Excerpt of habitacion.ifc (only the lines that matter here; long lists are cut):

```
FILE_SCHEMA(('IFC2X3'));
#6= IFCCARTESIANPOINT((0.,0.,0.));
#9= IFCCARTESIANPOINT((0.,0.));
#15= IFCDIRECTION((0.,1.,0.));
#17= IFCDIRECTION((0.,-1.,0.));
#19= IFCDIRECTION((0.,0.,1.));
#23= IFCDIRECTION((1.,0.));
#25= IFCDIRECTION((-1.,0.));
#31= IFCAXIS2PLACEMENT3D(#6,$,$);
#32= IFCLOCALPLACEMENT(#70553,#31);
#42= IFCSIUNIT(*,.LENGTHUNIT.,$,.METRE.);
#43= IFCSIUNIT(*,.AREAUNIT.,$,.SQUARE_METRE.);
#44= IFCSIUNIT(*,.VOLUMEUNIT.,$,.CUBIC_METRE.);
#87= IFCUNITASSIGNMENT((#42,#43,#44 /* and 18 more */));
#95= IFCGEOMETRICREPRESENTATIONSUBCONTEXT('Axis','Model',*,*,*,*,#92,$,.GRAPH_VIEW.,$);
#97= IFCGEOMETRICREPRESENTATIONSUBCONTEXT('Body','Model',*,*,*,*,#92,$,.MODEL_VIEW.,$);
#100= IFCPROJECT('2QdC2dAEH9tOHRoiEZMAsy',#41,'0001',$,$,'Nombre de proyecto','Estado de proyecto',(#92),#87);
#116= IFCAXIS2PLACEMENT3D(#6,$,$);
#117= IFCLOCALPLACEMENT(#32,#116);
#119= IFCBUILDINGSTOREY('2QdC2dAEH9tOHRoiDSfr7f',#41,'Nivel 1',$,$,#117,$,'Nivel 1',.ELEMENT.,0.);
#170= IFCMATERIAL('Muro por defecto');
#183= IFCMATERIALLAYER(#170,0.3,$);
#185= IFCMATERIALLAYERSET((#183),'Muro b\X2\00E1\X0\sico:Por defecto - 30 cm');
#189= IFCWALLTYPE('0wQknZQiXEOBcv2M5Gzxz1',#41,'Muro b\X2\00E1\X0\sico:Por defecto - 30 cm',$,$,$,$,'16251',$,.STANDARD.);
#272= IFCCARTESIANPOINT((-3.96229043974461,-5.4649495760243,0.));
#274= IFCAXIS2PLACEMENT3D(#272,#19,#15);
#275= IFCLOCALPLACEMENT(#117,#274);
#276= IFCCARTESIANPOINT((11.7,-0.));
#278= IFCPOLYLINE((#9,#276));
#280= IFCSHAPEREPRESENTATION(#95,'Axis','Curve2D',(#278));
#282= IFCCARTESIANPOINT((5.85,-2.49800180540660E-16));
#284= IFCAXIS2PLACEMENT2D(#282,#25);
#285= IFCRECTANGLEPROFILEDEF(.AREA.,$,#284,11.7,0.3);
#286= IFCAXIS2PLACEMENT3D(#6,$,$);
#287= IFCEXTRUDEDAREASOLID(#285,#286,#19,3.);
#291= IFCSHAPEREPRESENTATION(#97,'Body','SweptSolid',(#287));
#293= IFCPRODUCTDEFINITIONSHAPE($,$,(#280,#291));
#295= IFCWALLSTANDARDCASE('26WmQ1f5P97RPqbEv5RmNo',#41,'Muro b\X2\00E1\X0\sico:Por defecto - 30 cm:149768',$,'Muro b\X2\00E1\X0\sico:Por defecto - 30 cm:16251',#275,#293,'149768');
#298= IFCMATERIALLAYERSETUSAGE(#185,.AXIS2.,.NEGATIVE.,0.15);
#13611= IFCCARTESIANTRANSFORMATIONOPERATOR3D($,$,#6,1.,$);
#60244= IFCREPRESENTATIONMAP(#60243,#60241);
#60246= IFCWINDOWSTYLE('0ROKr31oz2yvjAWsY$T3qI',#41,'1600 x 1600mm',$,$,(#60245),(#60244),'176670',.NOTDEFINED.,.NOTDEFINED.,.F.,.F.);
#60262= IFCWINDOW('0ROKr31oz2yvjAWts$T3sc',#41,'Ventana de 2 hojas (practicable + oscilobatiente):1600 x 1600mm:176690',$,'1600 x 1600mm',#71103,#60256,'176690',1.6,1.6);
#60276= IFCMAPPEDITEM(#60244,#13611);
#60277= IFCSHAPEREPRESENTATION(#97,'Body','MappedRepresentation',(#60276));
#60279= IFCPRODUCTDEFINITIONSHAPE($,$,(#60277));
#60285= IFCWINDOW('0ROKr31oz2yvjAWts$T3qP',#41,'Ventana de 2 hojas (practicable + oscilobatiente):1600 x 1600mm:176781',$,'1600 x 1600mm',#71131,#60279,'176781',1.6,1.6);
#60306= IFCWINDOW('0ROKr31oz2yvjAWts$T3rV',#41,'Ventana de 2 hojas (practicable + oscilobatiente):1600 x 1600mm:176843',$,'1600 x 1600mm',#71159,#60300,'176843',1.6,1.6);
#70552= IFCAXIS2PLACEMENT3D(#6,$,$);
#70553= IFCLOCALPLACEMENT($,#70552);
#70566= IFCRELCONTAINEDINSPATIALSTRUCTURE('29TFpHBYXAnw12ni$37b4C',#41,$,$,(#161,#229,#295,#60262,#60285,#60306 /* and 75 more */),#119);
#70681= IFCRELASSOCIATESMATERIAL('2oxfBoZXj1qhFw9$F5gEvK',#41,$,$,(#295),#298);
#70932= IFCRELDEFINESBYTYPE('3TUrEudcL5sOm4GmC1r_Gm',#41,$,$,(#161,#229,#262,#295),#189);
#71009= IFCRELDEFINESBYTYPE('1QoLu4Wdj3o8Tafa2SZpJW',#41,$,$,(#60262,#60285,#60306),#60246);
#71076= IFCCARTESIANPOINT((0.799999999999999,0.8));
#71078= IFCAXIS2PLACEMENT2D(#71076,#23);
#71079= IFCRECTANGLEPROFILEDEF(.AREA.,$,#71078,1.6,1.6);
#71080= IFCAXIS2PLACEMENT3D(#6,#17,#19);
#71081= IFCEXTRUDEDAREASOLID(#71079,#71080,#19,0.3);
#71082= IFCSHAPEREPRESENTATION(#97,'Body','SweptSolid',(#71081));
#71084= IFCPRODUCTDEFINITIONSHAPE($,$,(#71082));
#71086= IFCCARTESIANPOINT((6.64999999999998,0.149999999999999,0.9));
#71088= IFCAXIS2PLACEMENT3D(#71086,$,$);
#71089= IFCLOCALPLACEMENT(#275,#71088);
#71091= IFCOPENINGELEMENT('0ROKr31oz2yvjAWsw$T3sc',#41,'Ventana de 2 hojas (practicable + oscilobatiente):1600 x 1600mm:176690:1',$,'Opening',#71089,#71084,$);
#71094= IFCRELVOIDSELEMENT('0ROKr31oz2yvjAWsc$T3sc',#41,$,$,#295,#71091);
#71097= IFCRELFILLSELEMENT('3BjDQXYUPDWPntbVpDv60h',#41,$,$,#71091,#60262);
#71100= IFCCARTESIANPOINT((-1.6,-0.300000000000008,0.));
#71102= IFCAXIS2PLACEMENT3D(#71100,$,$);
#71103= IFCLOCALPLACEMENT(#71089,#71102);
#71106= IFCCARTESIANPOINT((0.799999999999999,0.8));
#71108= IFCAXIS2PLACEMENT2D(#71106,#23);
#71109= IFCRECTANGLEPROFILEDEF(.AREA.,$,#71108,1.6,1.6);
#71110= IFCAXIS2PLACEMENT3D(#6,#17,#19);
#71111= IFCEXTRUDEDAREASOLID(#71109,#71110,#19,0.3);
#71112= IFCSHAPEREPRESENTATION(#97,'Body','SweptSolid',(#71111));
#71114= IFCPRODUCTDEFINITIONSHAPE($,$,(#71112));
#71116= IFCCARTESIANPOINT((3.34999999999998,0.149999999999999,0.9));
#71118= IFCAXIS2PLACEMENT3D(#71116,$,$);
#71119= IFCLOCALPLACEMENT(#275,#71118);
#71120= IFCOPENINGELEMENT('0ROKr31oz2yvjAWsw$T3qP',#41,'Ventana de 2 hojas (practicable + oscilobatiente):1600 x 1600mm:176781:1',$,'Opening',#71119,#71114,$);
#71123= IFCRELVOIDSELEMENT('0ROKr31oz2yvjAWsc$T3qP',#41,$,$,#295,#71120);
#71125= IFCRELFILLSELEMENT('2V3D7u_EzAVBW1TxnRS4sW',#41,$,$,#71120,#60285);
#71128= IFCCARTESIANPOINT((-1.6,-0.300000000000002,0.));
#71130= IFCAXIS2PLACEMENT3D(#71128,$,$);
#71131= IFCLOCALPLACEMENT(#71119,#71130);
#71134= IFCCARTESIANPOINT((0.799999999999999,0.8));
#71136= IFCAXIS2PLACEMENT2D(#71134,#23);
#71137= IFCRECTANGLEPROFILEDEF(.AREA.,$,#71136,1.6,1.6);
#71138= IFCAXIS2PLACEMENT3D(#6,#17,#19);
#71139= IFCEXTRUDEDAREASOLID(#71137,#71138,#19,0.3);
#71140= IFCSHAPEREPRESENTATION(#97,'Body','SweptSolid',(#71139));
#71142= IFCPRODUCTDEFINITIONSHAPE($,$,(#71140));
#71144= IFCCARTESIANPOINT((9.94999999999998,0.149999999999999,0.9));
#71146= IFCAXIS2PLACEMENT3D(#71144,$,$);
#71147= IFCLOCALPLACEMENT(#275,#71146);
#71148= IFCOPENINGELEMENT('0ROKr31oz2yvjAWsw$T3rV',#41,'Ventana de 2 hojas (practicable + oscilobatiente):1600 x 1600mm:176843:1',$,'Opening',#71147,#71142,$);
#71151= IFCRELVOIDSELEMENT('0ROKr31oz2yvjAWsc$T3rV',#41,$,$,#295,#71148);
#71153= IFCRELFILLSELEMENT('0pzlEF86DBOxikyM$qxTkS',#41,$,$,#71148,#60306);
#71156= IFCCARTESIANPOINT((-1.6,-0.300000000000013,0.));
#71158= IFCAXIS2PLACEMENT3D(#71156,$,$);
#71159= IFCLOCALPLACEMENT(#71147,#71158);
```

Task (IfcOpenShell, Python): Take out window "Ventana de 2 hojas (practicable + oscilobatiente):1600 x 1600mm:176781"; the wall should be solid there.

```python
import ifcopenshell
import ifcopenshell.api.feature
import ifcopenshell.api.root
import ifcopenshell.geom
import ifcopenshell.util.shape

model = ifcopenshell.open("habitacion.ifc")
settings = ifcopenshell.geom.settings()


def volume(element):
    """Net volume in cubic metres, openings subtracted."""
    shape = ifcopenshell.geom.create_shape(settings, element)
    return ifcopenshell.util.shape.get_volume(shape.geometry)


window = model.by_id(60285)
opening = window.FillsVoids[0].RelatingOpeningElement
wall = opening.VoidsElements[0].RelatingBuildingElement
before = volume(wall)

ifcopenshell.api.root.remove_product(model, product=window)
ifcopenshell.api.feature.remove_feature(model, feature=opening)

after = volume(wall)

print(f"wall volume {before:.3f} -> {after:.3f} m3")

model.write("habitacion_edited.ifc")
```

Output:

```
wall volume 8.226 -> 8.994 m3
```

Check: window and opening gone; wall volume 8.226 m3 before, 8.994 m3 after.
